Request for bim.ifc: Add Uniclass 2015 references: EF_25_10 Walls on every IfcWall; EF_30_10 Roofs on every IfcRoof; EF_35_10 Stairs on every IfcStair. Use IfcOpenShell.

First a look at what the model holds.

```python
import ifcopenshell

model = ifcopenshell.open("bim.ifc")
print(model.schema)
print("classifications:", [c.Name for c in model.by_type("IfcClassification")])
for ifc_class in ("IfcDoor", "IfcRoof", "IfcStair", "IfcWall", "IfcWindow"):
    print(ifc_class, len(model.by_type(ifc_class)))
```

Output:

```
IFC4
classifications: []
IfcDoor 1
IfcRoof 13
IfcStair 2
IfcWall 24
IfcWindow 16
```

```python
import ifcopenshell
import ifcopenshell.api.classification

model = ifcopenshell.open("bim.ifc")

system = ifcopenshell.api.classification.add_classification(model, classification="Uniclass 2015")

codes = {
    "IfcWall": ("EF_25_10", "Walls"),
    "IfcRoof": ("EF_30_10", "Roofs"),
    "IfcStair": ("EF_35_10", "Stairs"),
}
for ifc_class, (code, name) in codes.items():
    products = model.by_type(ifc_class)
    ifcopenshell.api.classification.add_reference(
        model, products=products, classification=system, identification=code, name=name
    )
    print(code, len(products))

model.write("bim_rev.ifc")
```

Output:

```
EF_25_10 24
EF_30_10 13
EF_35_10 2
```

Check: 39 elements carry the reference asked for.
